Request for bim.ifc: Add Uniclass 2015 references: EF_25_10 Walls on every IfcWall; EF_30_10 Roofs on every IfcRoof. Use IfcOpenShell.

First a look at what the model holds.

```python
import ifcopenshell

model = ifcopenshell.open("bim.ifc")
print(model.schema)
print("classifications:", [c.Name for c in model.by_type("IfcClassification")])
for ifc_class in ("IfcDoor", "IfcRoof", "IfcStair", "IfcWall", "IfcWindow"):
    print(ifc_class, len(model.by_type(ifc_class)))
```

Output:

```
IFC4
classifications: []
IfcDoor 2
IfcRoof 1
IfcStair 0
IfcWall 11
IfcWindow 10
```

```python
import ifcopenshell
import ifcopenshell.api.classification

model = ifcopenshell.open("bim.ifc")

system = ifcopenshell.api.classification.add_classification(model, classification="Uniclass 2015")

codes = {
    "IfcWall": ("EF_25_10", "Walls"),
    "IfcRoof": ("EF_30_10", "Roofs"),
}
for ifc_class, (code, name) in codes.items():
    products = model.by_type(ifc_class)
    ifcopenshell.api.classification.add_reference(
        model, products=products, classification=system, identification=code, name=name
    )
    print(code, len(products))

model.write("bim_updated.ifc")
```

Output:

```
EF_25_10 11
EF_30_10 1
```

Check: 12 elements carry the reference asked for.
